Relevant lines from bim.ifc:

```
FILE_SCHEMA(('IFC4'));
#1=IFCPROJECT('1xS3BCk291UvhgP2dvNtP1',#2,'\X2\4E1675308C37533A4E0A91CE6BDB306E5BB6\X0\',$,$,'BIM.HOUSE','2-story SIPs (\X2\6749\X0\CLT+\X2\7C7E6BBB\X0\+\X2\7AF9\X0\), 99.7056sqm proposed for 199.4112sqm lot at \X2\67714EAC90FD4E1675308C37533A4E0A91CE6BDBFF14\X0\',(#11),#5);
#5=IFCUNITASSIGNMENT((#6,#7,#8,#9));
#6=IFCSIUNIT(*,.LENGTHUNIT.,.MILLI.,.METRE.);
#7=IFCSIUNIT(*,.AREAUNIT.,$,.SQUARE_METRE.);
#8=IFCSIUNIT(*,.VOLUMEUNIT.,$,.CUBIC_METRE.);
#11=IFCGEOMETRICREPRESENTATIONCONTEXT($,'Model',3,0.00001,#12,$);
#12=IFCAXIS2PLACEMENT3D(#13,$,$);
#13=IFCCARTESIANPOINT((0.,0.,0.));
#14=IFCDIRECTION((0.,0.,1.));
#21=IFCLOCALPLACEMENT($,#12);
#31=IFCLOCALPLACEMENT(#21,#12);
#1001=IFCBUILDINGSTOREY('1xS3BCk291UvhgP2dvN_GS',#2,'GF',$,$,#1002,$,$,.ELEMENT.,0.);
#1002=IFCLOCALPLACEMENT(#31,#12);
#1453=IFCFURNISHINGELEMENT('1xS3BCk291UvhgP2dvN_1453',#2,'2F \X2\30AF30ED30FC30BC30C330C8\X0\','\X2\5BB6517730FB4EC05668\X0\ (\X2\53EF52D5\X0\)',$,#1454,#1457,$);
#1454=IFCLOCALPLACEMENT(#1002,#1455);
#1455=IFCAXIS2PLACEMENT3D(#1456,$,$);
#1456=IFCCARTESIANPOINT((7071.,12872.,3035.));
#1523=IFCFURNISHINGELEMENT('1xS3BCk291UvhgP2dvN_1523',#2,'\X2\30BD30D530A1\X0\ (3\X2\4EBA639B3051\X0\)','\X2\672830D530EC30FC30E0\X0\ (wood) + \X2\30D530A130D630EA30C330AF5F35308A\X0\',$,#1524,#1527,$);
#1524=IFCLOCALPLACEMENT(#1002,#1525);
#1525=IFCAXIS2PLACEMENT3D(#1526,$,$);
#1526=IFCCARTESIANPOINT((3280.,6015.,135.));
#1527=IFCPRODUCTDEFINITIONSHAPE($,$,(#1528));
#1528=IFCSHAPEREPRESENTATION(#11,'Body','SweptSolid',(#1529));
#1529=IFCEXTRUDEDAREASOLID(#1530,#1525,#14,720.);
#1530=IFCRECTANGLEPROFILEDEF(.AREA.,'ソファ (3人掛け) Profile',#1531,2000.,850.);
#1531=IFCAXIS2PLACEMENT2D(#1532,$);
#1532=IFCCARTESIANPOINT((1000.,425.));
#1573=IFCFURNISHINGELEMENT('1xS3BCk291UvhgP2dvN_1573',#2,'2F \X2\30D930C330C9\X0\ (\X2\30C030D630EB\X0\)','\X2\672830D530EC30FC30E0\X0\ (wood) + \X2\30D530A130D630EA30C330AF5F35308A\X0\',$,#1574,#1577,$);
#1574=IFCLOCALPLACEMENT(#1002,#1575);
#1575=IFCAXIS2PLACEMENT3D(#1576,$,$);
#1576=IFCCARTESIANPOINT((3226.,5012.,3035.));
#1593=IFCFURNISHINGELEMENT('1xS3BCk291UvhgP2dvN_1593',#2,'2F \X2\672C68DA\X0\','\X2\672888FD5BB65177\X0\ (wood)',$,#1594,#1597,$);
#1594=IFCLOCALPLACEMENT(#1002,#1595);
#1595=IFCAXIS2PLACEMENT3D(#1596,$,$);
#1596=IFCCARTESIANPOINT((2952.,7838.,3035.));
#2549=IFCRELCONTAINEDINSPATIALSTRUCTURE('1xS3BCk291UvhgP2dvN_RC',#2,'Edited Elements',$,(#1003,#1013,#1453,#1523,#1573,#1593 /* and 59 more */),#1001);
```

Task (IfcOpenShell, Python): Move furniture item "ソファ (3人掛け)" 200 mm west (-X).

```python
import ifcopenshell
import ifcopenshell.api.geometry
import ifcopenshell.util.placement
import ifcopenshell.util.unit

model = ifcopenshell.open("bim.ifc")
unit_scale = ifcopenshell.util.unit.calculate_unit_scale(model)

item = model.by_guid("1xS3BCk291UvhgP2dvN_1523")
matrix = ifcopenshell.util.placement.get_local_placement(item.ObjectPlacement)
matrix[0, 3] -= 0.2 / unit_scale
ifcopenshell.api.geometry.edit_object_placement(model, product=item, matrix=matrix, is_si=False)

print(ifcopenshell.util.placement.get_local_placement(item.ObjectPlacement).round(3) + 0.0)

model.write("bim_edited.ifc")
```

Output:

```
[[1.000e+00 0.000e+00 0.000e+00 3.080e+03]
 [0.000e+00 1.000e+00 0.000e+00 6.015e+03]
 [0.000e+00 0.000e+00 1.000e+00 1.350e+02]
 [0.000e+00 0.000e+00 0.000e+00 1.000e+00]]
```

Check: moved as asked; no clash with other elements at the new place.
